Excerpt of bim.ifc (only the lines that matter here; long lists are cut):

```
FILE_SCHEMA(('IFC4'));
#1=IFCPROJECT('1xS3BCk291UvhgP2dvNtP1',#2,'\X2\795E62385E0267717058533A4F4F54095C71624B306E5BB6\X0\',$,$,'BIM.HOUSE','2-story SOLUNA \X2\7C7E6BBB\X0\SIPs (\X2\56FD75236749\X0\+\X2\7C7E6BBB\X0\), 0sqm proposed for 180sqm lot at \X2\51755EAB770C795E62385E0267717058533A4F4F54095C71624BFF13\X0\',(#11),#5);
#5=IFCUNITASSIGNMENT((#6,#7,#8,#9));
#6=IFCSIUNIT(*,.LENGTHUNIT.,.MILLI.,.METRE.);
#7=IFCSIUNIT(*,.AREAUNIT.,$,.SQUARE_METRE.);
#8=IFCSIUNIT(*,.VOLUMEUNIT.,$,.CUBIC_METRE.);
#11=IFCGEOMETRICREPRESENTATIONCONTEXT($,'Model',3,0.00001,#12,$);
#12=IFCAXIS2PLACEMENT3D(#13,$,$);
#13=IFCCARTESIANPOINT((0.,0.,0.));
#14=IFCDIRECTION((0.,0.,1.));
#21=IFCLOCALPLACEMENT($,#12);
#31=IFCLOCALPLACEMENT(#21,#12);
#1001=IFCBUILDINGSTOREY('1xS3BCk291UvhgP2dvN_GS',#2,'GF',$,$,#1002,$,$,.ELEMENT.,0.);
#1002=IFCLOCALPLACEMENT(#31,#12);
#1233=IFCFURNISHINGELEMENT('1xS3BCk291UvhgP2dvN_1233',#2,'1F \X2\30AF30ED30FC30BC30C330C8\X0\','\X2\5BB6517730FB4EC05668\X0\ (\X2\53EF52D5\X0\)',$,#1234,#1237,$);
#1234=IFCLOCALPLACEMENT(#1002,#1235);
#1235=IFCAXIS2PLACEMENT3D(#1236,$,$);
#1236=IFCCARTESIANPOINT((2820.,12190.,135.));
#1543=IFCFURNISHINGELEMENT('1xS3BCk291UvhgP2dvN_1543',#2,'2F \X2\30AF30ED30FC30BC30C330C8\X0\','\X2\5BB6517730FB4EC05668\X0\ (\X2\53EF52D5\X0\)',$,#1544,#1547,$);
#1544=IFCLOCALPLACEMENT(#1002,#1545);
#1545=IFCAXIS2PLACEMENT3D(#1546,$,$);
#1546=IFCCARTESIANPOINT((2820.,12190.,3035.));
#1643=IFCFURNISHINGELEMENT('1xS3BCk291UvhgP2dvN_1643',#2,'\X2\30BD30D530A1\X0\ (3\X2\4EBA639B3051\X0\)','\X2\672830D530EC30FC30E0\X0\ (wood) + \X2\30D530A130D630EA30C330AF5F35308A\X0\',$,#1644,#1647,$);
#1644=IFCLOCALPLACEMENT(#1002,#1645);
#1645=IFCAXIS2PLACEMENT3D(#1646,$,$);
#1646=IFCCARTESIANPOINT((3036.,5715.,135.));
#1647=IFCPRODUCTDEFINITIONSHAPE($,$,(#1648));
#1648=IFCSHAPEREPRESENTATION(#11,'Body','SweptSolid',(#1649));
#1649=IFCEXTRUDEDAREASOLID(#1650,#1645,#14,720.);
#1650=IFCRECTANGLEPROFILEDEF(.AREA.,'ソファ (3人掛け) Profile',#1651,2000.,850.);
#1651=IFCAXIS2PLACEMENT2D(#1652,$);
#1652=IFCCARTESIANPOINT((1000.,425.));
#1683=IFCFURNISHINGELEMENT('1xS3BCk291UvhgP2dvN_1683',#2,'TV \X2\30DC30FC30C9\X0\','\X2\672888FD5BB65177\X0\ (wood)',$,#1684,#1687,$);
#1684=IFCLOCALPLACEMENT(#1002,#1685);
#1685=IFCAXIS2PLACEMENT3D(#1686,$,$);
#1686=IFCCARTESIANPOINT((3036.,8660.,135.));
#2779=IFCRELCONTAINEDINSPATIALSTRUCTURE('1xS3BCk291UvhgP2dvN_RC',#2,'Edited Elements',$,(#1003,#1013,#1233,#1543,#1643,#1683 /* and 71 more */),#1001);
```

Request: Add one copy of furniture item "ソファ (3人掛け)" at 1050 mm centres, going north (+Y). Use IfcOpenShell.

```python
import numpy as np
import ifcopenshell
import ifcopenshell.api.geometry
import ifcopenshell.api.root
import ifcopenshell.util.element
import ifcopenshell.util.placement
import ifcopenshell.util.unit

model = ifcopenshell.open("bim.ifc")
unit_scale = ifcopenshell.util.unit.calculate_unit_scale(model)


def reuse_history(source, copy):
    """copy_class also copies each property set's owner history, people and application; keep the originals."""
    for rel in copy.IsDefinedBy:
        if rel.is_a("IfcRelDefinesByProperties") and (history := rel.RelatingPropertyDefinition.OwnerHistory):
            rel.RelatingPropertyDefinition.OwnerHistory = source.OwnerHistory
            ifcopenshell.util.element.remove_deep2(model, history)


source = model.by_guid("1xS3BCk291UvhgP2dvN_1643")
base = ifcopenshell.util.placement.get_local_placement(source.ObjectPlacement)
step = np.array([0.0, 1.0, 0.0]) * 1.05 / unit_scale

for i in range(1, 2):
    copy = ifcopenshell.api.root.copy_class(model, product=source)
    copy.Representation = ifcopenshell.util.element.copy_deep(
        model, source.Representation, exclude=["IfcGeometricRepresentationContext", "IfcRepresentationMap"]
    )
    reuse_history(source, copy)
    matrix = base.copy()
    matrix[:3, 3] += i * step
    print("added at", matrix[:3, 3].round(3) + 0.0)
    ifcopenshell.api.geometry.edit_object_placement(model, product=copy, matrix=matrix, is_si=False)

model.write("bim_edited.ifc")
```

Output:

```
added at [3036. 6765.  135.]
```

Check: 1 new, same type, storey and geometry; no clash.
